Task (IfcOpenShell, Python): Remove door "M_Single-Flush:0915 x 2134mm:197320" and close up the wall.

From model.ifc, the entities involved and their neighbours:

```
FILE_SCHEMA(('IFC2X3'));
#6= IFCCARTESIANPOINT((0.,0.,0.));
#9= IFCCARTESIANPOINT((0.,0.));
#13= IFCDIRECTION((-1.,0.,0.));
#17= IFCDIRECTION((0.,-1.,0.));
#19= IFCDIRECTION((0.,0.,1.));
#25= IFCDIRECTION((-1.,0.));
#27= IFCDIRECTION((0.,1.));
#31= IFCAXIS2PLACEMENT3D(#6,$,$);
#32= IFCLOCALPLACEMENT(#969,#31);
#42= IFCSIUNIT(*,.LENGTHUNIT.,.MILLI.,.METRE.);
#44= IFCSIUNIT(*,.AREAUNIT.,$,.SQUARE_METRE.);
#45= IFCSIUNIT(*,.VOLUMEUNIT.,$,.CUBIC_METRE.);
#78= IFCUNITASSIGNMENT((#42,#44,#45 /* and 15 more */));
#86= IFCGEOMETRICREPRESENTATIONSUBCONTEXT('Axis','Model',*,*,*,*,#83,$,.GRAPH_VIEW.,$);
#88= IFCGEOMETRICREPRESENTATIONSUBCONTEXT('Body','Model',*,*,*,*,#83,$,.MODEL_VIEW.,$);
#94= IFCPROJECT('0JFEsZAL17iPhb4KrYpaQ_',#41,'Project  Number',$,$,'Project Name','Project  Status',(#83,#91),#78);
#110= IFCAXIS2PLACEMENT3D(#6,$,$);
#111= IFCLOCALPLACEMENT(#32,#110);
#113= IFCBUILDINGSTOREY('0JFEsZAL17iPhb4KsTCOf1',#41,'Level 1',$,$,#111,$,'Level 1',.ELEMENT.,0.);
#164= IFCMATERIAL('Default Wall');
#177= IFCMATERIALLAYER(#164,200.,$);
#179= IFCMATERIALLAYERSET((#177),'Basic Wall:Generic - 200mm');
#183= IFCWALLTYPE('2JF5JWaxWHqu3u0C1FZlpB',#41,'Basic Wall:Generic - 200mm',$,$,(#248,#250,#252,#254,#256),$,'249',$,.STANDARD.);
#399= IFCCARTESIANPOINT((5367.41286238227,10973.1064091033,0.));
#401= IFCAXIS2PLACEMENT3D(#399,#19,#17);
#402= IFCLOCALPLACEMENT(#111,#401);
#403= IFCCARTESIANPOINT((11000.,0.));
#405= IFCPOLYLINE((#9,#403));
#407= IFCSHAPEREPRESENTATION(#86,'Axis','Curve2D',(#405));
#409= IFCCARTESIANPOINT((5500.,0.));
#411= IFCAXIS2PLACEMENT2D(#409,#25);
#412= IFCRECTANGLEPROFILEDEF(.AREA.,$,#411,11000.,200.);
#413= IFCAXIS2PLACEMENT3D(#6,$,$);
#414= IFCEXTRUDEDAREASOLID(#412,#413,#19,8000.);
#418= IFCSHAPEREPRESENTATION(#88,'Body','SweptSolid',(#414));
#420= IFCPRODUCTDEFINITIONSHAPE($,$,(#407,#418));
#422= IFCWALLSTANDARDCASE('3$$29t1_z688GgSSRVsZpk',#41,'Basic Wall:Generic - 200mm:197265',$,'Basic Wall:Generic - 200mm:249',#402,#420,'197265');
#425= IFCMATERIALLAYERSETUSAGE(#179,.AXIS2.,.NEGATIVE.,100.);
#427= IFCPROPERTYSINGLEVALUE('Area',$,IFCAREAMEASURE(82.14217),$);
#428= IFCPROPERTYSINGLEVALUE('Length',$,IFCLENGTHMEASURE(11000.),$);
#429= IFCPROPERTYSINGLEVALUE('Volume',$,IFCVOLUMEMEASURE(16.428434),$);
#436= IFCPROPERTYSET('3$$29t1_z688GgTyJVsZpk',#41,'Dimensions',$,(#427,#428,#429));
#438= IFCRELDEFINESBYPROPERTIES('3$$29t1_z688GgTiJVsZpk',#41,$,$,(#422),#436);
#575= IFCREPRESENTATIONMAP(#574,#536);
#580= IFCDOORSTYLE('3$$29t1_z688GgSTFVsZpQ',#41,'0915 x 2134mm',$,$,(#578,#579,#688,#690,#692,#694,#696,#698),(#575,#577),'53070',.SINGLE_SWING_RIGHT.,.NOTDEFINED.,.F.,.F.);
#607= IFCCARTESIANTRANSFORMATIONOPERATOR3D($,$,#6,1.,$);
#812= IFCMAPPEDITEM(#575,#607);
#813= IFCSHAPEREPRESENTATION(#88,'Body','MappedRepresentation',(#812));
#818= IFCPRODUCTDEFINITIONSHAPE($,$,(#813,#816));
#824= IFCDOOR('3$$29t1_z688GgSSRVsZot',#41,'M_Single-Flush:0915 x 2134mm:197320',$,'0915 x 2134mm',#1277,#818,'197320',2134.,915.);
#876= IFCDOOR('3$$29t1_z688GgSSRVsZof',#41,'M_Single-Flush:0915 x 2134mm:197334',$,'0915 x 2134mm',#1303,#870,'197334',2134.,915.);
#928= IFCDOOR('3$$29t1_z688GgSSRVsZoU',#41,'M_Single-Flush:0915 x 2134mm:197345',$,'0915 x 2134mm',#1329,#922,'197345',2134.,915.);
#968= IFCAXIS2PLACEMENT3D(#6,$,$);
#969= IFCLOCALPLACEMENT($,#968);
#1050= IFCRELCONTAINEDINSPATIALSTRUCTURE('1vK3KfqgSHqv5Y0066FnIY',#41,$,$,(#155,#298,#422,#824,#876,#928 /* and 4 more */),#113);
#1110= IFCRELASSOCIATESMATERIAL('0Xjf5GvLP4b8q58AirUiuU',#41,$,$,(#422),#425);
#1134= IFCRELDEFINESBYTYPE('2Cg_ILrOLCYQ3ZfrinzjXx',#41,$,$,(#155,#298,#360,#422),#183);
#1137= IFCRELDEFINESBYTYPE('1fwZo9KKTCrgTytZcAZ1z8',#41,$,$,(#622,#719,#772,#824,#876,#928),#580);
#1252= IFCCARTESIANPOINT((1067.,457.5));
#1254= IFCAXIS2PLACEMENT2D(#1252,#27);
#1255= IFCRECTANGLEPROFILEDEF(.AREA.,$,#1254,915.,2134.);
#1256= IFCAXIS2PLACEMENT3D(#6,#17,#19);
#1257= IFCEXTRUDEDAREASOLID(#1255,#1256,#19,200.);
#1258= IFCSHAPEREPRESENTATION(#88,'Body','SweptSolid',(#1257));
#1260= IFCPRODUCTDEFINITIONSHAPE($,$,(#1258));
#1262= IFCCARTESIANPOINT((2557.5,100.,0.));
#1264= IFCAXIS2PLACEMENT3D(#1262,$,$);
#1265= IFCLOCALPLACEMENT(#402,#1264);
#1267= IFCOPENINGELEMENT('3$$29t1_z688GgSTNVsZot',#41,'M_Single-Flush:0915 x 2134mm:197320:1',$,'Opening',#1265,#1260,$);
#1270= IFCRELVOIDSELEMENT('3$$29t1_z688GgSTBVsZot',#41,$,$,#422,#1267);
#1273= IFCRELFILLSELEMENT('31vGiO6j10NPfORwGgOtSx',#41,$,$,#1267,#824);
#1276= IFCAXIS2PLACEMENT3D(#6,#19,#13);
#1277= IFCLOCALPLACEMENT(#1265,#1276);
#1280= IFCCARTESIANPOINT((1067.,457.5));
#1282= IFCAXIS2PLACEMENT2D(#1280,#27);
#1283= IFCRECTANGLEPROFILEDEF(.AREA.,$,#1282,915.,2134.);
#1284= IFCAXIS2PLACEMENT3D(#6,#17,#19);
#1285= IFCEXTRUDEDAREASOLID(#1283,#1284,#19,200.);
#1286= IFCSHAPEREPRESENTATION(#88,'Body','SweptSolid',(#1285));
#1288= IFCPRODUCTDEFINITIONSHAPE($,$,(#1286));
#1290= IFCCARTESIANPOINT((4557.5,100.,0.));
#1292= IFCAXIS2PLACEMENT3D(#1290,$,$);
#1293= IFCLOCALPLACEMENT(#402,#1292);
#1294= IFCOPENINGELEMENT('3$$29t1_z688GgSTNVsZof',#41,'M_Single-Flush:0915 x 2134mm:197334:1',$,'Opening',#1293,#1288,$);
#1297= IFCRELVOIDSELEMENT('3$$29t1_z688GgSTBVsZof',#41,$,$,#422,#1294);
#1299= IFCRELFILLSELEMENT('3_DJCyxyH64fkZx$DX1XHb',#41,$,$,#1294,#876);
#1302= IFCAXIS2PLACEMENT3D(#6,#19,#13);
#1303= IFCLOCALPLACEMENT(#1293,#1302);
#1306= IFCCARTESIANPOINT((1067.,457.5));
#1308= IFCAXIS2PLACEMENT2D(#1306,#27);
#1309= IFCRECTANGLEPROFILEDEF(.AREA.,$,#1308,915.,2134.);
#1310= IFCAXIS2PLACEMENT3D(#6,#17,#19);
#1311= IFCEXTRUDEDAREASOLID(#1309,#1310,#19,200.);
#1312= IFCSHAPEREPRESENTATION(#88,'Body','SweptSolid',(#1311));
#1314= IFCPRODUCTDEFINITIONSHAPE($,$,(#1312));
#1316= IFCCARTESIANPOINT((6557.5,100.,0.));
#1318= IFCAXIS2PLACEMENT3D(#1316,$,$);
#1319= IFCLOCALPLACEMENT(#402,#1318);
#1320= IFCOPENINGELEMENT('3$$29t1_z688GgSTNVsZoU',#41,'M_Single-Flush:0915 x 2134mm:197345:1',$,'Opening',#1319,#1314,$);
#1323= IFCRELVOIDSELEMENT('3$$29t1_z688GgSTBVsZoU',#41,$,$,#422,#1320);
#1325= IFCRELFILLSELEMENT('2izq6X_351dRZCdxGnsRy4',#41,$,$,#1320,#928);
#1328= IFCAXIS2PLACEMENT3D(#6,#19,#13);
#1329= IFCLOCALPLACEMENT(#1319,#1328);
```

```python
import ifcopenshell
import ifcopenshell.api.feature
import ifcopenshell.api.pset
import ifcopenshell.api.root
import ifcopenshell.geom
import ifcopenshell.util.element
import ifcopenshell.util.shape
import ifcopenshell.util.unit

model = ifcopenshell.open("model.ifc")
area_scale = ifcopenshell.util.unit.calculate_unit_scale(model, "AREAUNIT")
volume_scale = ifcopenshell.util.unit.calculate_unit_scale(model, "VOLUMEUNIT")
settings = ifcopenshell.geom.settings()


def volume(element):
    """Net volume in cubic metres, openings subtracted."""
    shape = ifcopenshell.geom.create_shape(settings, element)
    return ifcopenshell.util.shape.get_volume(shape.geometry)


door = model.by_id(824)
opening = door.FillsVoids[0].RelatingOpeningElement
wall = opening.VoidsElements[0].RelatingBuildingElement
before = volume(wall)

ifcopenshell.api.root.remove_product(model, product=door)
ifcopenshell.api.feature.remove_feature(model, feature=opening)

after = volume(wall)
thickness = 0.2  # wall thickness in metres

# Update the wall's stored quantities.
pset = model.by_id(ifcopenshell.util.element.get_pset(wall, "Dimensions", should_inherit=False)["id"])
ifcopenshell.api.pset.edit_pset(model, pset=pset, properties={
    "Area": model.create_entity("IfcAreaMeasure", after / thickness / area_scale),
    "Volume": model.create_entity("IfcVolumeMeasure", after / volume_scale),
})

print(f"wall volume {before:.3f} -> {after:.3f} m3")

model.write("model_v2.ifc")
```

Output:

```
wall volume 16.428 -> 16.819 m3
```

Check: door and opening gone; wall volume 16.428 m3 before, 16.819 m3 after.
